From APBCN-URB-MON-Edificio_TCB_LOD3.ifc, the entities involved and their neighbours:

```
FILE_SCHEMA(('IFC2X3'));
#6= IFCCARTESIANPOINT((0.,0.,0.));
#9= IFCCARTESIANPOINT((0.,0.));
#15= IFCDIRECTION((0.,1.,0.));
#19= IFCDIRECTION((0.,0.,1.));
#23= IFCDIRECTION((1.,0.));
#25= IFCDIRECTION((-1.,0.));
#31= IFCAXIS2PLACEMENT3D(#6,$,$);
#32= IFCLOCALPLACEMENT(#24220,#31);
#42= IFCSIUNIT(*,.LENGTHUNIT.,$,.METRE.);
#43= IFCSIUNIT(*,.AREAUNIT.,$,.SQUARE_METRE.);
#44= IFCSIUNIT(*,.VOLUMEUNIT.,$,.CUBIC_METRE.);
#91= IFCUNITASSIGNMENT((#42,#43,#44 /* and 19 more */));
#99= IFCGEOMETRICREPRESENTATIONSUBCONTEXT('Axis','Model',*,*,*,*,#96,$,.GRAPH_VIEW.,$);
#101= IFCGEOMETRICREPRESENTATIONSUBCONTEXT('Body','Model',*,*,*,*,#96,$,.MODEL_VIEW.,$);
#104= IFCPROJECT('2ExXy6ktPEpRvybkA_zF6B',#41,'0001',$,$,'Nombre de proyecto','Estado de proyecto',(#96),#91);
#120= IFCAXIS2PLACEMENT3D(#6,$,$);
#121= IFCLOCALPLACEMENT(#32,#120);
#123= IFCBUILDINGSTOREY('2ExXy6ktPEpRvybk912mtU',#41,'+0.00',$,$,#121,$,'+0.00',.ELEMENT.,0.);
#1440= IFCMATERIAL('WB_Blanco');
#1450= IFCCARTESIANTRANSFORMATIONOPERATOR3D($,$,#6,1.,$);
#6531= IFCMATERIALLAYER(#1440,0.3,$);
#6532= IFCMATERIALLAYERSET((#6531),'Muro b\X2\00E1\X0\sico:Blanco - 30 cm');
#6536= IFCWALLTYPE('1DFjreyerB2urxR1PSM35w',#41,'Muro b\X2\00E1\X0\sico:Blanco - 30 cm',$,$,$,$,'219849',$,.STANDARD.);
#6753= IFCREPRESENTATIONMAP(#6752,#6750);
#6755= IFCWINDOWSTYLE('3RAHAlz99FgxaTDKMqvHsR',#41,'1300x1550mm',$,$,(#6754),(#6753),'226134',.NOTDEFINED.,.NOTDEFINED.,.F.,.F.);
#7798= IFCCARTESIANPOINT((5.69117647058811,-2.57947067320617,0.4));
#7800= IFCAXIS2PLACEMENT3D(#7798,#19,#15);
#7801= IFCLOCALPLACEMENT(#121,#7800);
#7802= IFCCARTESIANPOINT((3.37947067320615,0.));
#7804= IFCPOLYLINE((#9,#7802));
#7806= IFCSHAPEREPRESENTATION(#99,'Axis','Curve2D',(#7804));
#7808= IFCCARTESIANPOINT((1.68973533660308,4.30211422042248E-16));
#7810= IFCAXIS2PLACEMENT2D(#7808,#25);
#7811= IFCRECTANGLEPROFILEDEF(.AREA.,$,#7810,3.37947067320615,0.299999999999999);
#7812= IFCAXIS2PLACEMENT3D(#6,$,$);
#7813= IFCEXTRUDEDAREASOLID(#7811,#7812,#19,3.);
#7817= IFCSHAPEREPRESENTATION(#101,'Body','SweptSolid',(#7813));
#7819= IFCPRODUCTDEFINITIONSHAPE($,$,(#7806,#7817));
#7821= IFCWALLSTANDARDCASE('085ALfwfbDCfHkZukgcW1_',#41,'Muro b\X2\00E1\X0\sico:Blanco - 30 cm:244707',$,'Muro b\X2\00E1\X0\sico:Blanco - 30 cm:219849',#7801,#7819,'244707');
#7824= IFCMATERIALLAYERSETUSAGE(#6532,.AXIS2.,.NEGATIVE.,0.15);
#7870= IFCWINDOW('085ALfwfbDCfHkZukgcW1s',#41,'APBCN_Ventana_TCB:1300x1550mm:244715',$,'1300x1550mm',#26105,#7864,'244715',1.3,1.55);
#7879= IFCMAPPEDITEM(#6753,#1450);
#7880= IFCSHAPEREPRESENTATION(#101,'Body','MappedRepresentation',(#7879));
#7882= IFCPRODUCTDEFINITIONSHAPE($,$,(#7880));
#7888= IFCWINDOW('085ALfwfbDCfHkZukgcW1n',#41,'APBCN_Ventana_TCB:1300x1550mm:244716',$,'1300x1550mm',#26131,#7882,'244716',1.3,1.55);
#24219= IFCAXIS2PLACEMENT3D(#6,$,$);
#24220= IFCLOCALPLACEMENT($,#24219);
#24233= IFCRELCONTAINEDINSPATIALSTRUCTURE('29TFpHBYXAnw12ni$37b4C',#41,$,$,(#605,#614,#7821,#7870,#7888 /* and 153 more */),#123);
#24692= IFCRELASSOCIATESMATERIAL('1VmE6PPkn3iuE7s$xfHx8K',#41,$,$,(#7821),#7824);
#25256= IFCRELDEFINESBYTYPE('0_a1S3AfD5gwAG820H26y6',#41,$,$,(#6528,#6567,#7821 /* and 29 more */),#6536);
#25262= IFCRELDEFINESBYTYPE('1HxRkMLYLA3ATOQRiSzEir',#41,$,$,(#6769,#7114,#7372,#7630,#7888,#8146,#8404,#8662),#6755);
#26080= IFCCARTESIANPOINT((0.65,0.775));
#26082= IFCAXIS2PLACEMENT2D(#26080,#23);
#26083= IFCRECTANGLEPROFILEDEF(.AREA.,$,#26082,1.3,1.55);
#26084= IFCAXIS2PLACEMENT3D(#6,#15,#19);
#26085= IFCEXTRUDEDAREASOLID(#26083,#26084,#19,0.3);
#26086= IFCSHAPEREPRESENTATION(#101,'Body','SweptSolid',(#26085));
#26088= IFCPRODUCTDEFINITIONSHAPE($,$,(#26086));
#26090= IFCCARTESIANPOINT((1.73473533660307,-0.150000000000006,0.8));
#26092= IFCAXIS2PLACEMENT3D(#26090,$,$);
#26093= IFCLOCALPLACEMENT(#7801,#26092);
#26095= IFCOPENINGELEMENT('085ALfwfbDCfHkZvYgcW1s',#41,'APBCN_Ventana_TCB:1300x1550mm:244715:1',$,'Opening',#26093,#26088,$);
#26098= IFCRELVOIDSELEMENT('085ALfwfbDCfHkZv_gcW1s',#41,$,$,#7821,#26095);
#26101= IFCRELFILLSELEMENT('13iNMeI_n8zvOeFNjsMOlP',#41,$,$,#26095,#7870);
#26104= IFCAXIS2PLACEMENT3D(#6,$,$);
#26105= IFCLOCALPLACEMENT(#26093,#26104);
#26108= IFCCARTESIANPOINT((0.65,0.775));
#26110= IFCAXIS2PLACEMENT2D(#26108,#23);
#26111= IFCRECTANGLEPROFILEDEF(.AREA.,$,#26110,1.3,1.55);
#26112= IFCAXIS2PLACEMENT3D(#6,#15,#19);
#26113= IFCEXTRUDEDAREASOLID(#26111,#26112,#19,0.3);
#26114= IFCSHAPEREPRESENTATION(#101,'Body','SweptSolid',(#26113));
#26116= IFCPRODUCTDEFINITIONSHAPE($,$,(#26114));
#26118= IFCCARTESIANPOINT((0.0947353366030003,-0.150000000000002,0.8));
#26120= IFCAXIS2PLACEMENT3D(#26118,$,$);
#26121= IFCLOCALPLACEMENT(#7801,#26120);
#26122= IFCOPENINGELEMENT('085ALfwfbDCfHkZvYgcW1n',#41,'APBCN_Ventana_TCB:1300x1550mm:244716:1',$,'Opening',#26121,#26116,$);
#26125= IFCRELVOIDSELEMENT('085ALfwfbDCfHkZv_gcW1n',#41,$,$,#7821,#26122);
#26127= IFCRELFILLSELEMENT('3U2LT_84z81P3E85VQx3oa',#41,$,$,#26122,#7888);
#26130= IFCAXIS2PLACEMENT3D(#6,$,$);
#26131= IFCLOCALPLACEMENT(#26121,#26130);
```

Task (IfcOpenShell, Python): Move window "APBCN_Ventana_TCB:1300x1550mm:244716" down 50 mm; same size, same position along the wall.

```python
import numpy as np
import ifcopenshell
import ifcopenshell.api.geometry
import ifcopenshell.util.placement
import ifcopenshell.util.unit

model = ifcopenshell.open("APBCN-URB-MON-Edificio_TCB_LOD3.ifc")
unit_scale = ifcopenshell.util.unit.calculate_unit_scale(model)

window = model.by_guid("085ALfwfbDCfHkZukgcW1n")
opening = window.FillsVoids[0].RelatingOpeningElement
dz = -0.05 / unit_scale

shift = np.array([0.0, 0.0, dz])
# The window is placed relative to its opening, so it follows when the opening moves.
matrix = ifcopenshell.util.placement.get_local_placement(opening.ObjectPlacement)
matrix[:3, 3] += shift
ifcopenshell.api.geometry.edit_object_placement(
    model, product=opening, matrix=matrix, is_si=False, should_transform_children=True
)

print(f"moved by {dz * unit_scale:+.3f} m")

model.write("APBCN-URB-MON-Edificio_TCB_LOD3_updated.ifc")
```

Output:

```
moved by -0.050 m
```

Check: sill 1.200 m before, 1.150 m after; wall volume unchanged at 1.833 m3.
